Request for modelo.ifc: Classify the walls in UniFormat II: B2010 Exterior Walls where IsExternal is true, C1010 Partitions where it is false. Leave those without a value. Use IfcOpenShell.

First a look at what the model holds.

```python
import ifcopenshell
import ifcopenshell.util.element

model = ifcopenshell.open("modelo.ifc")
print(model.schema)
print("classifications:", [c.Name for c in model.by_type("IfcClassification")])
values = [ifcopenshell.util.element.get_pset(e, "Pset_WallCommon", "IsExternal") for e in model.by_type("IfcWall")]
for value in (True, False, None):
    print("IsExternal", value, values.count(value))
```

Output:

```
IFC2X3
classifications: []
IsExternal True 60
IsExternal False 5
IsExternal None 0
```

```python
import ifcopenshell
import ifcopenshell.api.classification
import ifcopenshell.util.element

model = ifcopenshell.open("modelo.ifc")

# IFC2X3 requires Source and Edition and has no link from the project to the system.
system = model.create_entity("IfcClassification", Source="ASTM", Edition="E1557", Name="UniFormat II")

walls = model.by_type("IfcWall")
external = {e: ifcopenshell.util.element.get_pset(e, "Pset_WallCommon", "IsExternal") for e in walls}
for flag, code, name in ((True, "B2010", "Exterior Walls"), (False, "C1010", "Partitions")):
    products = [e for e in walls if external[e] is flag]
    ifcopenshell.api.classification.add_reference(
        model, products=products, classification=system, identification=code, name=name
    )
    print(code, len(products))

model.write("modelo_updated.ifc")
```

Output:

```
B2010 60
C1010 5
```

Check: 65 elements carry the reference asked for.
